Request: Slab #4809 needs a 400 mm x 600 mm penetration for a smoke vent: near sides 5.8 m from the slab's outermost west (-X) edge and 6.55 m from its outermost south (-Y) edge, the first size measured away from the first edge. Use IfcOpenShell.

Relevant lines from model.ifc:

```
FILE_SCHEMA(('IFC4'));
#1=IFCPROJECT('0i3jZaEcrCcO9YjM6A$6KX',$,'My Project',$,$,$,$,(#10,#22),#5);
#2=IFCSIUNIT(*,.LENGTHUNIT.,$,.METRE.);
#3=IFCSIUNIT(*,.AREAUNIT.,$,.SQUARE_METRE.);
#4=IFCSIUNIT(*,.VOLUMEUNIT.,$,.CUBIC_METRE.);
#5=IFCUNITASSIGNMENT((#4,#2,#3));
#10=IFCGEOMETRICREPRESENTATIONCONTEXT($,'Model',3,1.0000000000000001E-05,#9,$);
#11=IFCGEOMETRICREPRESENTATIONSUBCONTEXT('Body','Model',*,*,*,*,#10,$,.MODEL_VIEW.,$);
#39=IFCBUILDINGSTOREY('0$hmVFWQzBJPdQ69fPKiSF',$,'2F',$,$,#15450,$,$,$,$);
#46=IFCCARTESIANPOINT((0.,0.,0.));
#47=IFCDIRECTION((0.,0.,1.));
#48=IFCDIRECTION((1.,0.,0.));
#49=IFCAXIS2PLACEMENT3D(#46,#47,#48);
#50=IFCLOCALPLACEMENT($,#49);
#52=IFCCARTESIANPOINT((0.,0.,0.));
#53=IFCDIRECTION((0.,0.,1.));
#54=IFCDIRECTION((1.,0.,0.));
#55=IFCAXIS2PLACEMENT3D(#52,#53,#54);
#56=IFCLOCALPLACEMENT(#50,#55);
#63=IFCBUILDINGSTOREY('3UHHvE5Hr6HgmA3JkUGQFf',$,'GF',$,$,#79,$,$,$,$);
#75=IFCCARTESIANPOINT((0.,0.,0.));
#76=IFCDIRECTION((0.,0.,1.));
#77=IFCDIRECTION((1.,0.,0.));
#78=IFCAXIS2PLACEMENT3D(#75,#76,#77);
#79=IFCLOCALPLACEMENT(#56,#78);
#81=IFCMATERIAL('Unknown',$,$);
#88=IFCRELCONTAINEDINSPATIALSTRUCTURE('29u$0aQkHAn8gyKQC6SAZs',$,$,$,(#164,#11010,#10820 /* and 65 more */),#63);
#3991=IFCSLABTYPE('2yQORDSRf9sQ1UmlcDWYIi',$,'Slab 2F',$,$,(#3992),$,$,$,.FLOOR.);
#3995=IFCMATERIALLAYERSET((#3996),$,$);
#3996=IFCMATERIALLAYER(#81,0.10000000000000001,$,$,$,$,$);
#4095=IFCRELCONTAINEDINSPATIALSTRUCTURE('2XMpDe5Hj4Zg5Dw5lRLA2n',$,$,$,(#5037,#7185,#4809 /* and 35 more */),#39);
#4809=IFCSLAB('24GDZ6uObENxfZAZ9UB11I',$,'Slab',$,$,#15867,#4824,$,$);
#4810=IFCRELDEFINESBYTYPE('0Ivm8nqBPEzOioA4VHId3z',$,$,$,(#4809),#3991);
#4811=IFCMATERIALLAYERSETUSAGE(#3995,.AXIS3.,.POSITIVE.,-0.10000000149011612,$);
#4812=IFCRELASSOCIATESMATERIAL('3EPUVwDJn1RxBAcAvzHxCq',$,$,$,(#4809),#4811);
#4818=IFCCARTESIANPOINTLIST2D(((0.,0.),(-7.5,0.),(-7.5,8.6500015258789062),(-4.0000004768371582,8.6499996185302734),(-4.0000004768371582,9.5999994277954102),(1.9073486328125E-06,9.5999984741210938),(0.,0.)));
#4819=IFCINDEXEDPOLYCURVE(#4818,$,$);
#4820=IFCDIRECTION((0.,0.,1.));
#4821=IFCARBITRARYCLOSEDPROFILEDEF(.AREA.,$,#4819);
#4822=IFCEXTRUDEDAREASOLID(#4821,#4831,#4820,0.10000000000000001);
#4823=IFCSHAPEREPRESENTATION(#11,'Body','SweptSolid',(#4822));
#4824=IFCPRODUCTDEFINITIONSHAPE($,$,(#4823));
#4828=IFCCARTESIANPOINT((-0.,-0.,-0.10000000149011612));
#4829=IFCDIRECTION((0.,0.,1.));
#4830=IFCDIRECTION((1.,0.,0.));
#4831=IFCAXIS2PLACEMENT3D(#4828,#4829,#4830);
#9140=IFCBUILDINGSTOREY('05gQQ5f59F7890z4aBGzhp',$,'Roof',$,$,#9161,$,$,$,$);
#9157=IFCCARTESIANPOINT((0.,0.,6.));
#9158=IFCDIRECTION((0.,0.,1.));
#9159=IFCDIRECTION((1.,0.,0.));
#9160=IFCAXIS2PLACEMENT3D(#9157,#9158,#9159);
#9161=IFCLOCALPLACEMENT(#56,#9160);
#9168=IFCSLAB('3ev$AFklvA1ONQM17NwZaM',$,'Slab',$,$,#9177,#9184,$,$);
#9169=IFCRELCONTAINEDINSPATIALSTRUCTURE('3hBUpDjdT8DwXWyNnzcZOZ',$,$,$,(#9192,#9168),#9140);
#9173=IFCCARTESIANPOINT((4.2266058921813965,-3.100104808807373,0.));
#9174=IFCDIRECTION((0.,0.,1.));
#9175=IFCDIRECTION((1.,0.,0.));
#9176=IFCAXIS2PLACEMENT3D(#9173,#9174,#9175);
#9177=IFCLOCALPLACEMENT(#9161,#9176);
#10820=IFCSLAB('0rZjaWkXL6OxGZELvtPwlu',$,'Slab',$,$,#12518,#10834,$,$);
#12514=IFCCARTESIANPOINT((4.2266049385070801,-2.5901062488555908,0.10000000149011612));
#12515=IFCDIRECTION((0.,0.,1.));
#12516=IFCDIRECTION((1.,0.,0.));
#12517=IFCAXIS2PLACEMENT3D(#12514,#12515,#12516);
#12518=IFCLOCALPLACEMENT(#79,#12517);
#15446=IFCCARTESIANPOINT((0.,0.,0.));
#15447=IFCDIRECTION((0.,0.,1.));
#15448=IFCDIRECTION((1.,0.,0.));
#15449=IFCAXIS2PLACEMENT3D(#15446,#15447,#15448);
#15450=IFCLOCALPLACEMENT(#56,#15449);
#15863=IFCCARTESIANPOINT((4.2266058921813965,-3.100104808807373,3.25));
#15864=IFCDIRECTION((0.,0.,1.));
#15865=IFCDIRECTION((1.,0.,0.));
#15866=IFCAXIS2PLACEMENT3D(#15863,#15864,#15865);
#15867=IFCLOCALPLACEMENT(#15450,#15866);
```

```python
import numpy as np
import ifcopenshell
import ifcopenshell.api.feature
import ifcopenshell.api.geometry
import ifcopenshell.api.root
import ifcopenshell.geom
import ifcopenshell.util.placement
import ifcopenshell.util.representation
import ifcopenshell.util.shape
import ifcopenshell.util.unit

model = ifcopenshell.open("model.ifc")
unit_scale = ifcopenshell.util.unit.calculate_unit_scale(model)
settings = ifcopenshell.geom.settings()


def volume(element):
    """Net volume in cubic metres, openings subtracted."""
    shape = ifcopenshell.geom.create_shape(settings, element)
    return ifcopenshell.util.shape.get_volume(shape.geometry)


slab = model.by_guid("24GDZ6uObENxfZAZ9UB11I")
before = volume(slab)

# Extent in the slab's own axes, in metres. The edges named are its -X and -Y sides.
slab_shape = ifcopenshell.geom.create_shape(settings, slab)
vertices = ifcopenshell.util.shape.get_vertices(slab_shape.geometry)
x_min, y_min, bottom = vertices.min(axis=0)
top = vertices[:, 2].max()

opening = ifcopenshell.api.root.create_entity(model, ifc_class="IfcOpeningElement", name="Smoke vent opening", predefined_type="OPENING")
context = ifcopenshell.util.representation.get_context(model, "Model", "Body", "MODEL_VIEW")
width, depth = 0.4, 0.6
outline = [(0.0, 0.0), (width, 0.0), (width, depth), (0.0, depth), (0.0, 0.0)]
# Overshoot both faces by 50 mm so the cut is clean.
shape = ifcopenshell.api.geometry.add_slab_representation(
    model, context=context, depth=top - bottom + 0.1, polyline=outline
)
ifcopenshell.api.geometry.assign_representation(model, product=opening, representation=shape)

matrix = ifcopenshell.util.placement.get_local_placement(slab.ObjectPlacement)
matrix[:, 3] = matrix @ np.append(np.array([x_min + 5.8, y_min + 6.55, bottom - 0.05]) / unit_scale, 1.0)
ifcopenshell.api.geometry.edit_object_placement(model, product=opening, matrix=matrix, is_si=False)
ifcopenshell.api.feature.add_feature(model, feature=opening, element=slab)

after = volume(slab)

print(f"slab volume {before:.3f} -> {after:.3f} m3")

model.write("model_v2.ifc")
```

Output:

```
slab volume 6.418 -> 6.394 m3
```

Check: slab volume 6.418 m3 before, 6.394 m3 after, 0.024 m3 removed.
